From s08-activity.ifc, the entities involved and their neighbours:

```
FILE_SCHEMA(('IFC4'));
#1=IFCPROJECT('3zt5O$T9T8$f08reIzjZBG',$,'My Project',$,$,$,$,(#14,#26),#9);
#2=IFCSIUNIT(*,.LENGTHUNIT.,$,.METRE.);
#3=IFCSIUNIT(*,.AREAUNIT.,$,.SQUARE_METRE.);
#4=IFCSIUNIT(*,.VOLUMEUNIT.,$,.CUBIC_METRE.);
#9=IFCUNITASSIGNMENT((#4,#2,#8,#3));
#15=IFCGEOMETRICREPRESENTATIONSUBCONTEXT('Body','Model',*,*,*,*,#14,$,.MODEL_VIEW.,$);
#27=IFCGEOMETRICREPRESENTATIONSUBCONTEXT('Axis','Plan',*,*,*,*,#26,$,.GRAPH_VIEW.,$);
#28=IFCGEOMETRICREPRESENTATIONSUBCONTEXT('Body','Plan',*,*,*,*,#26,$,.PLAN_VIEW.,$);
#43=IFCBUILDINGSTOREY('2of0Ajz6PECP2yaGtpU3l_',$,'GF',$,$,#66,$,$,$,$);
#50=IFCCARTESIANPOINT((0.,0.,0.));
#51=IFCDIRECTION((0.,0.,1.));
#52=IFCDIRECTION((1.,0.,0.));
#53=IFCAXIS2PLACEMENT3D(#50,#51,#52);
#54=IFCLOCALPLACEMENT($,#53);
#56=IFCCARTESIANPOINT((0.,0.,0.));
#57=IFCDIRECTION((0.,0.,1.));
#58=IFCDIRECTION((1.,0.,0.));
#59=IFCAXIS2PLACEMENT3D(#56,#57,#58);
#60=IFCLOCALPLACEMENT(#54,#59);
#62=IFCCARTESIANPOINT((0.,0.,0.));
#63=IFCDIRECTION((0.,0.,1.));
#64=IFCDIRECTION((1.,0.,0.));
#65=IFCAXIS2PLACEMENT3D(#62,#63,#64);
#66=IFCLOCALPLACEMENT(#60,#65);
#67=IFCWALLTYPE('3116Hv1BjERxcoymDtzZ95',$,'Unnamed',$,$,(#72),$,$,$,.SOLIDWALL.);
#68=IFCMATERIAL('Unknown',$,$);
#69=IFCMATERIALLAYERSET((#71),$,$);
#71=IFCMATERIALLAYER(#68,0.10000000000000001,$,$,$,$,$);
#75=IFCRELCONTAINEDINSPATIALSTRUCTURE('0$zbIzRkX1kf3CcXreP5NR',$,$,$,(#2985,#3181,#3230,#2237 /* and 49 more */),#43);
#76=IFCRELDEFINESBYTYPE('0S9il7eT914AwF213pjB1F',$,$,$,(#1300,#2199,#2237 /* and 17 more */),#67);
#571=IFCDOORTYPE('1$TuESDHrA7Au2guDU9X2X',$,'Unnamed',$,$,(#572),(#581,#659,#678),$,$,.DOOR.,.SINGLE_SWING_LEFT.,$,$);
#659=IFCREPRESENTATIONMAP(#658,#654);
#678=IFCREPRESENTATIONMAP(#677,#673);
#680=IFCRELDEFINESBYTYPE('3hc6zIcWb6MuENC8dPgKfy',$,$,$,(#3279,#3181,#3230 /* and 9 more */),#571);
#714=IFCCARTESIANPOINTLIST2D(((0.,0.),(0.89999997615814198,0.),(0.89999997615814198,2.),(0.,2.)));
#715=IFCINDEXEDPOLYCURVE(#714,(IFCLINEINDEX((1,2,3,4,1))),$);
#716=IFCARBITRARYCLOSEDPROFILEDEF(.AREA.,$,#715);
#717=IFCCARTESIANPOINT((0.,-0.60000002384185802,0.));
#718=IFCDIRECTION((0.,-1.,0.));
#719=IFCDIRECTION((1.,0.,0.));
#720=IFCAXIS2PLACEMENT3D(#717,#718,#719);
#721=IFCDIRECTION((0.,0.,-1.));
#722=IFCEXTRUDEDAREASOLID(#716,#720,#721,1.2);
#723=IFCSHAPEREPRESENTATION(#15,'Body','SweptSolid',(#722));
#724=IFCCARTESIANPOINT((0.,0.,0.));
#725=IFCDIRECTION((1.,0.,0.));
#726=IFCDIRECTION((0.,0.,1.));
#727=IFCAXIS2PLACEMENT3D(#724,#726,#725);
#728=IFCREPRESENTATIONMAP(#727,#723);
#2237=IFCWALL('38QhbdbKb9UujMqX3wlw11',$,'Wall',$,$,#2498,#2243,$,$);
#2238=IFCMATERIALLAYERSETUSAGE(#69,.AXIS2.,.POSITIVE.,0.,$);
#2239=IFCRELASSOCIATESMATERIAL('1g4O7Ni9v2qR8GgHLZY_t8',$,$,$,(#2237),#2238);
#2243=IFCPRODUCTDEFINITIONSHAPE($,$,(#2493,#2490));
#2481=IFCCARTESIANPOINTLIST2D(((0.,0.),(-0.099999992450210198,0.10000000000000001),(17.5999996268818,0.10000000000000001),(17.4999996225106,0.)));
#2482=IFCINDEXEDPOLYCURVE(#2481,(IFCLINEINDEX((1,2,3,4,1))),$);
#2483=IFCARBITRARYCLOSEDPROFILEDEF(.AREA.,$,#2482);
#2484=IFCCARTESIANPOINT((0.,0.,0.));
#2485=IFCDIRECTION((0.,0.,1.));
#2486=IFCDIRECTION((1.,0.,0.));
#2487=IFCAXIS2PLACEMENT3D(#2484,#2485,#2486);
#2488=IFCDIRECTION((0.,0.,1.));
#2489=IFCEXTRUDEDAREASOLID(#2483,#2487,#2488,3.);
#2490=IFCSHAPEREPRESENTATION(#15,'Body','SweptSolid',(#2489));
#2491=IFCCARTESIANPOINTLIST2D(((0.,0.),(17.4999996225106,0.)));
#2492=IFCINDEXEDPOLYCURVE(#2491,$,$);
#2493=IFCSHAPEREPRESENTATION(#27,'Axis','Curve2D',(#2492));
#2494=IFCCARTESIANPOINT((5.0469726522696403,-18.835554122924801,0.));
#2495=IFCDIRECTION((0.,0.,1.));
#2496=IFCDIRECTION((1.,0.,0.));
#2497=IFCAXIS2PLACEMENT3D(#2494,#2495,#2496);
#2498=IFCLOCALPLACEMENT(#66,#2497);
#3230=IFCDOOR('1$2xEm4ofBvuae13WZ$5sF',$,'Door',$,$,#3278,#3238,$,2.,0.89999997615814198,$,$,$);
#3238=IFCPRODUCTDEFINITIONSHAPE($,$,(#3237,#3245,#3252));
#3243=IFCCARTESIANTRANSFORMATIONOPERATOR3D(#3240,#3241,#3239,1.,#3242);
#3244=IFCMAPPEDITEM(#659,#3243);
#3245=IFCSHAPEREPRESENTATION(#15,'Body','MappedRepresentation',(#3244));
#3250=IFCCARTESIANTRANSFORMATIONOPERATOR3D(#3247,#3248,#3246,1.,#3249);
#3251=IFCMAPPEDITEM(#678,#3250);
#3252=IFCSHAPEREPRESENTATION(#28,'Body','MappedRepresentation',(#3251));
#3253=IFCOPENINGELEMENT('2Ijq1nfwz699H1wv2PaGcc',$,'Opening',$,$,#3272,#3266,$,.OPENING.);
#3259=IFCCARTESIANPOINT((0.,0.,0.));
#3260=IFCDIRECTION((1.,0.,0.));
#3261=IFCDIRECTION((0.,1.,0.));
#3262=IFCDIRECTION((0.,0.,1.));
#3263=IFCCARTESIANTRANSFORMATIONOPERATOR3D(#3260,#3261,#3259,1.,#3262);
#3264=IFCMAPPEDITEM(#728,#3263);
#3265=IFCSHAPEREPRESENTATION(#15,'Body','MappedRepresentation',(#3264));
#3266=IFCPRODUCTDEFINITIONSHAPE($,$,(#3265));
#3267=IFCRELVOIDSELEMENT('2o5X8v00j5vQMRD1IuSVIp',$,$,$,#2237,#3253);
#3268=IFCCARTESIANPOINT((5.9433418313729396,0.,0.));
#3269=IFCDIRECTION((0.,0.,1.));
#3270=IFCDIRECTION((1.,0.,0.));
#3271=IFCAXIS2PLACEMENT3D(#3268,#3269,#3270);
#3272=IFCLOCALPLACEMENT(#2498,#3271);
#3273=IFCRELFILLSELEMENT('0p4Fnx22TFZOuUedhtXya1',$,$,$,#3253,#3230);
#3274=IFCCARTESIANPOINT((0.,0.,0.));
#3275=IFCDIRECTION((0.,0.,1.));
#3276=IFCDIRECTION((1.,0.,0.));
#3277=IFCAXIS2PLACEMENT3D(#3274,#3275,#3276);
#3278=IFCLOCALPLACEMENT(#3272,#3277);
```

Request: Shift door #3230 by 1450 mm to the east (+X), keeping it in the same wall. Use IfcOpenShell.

```python
import ifcopenshell
import ifcopenshell.api.geometry
import ifcopenshell.util.placement
import ifcopenshell.util.unit

model = ifcopenshell.open("s08-activity.ifc")
unit_scale = ifcopenshell.util.unit.calculate_unit_scale(model)

door = model.by_id(3230)
opening = door.FillsVoids[0].RelatingOpeningElement
wall = opening.VoidsElements[0].RelatingBuildingElement

wall_matrix = ifcopenshell.util.placement.get_local_placement(wall.ObjectPlacement)
shift = wall_matrix[:3, 0] * 1.45 / unit_scale
before = ifcopenshell.util.placement.get_local_placement(door.ObjectPlacement)[:3, 3].copy()

# The door is placed relative to its opening, so it follows when the opening moves.
matrix = ifcopenshell.util.placement.get_local_placement(opening.ObjectPlacement)
matrix[:3, 3] += shift
ifcopenshell.api.geometry.edit_object_placement(
    model, product=opening, matrix=matrix, is_si=False, should_transform_children=True
)

after = ifcopenshell.util.placement.get_local_placement(door.ObjectPlacement)[:3, 3]
print("door moved by", (after - before).round(3) + 0.0)

model.write("s08-activity-out.ifc")
```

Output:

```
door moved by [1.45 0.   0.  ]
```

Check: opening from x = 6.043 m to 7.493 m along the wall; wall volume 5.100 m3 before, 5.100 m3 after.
